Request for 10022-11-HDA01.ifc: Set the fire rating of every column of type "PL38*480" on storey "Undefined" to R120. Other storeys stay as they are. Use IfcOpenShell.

First a look at what the model holds.

```python
import ifcopenshell
import ifcopenshell.util.element

model = ifcopenshell.open("10022-11-HDA01.ifc")
print(model.schema)
storey = next(s for s in model.by_type("IfcBuildingStorey") if s.Name == "Undefined")
columns = [e for e in ifcopenshell.util.element.get_decomposition(storey) if e.is_a("IfcColumn")]
seen = {}
for e in columns:
    element_type = ifcopenshell.util.element.get_type(e)
    key = (element_type.Name if element_type != e and element_type else None, ifcopenshell.util.element.get_pset(e, "Pset_ColumnCommon", "FireRating"))
    seen[key] = seen.get(key, 0) + 1
for (name, value), count in sorted(seen.items(), key=str):
    print(count, "x", name, "|", value)
```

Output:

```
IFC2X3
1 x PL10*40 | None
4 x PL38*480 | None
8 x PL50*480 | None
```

```python
import ifcopenshell
import ifcopenshell.api.pset
import ifcopenshell.util.element

model = ifcopenshell.open("10022-11-HDA01.ifc")

storey = next(s for s in model.by_type("IfcBuildingStorey") if s.Name == "Undefined")
columns = [e for e in ifcopenshell.util.element.get_decomposition(storey) if e.is_a("IfcColumn")]

count = 0
for e in columns:
    element_type = ifcopenshell.util.element.get_type(e)
    if element_type in (None, e) or element_type.Name != "PL38*480":
        continue
    found = ifcopenshell.util.element.get_pset(e, "Pset_ColumnCommon", should_inherit=False)
    if found:
        pset = model.by_id(found["id"])
        if len(ifcopenshell.util.element.get_elements_by_pset(pset)) > 1:
            pset = ifcopenshell.api.pset.unshare_pset(model, products=[e], pset=pset)[0]
    else:
        pset = ifcopenshell.api.pset.add_pset(model, product=e, name="Pset_ColumnCommon")
    ifcopenshell.api.pset.edit_pset(model, pset=pset, properties={"FireRating": "R120"})
    count += 1

print(count, "columns updated")

model.write("10022-11-HDA01_edited.ifc")
```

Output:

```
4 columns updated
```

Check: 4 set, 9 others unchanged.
